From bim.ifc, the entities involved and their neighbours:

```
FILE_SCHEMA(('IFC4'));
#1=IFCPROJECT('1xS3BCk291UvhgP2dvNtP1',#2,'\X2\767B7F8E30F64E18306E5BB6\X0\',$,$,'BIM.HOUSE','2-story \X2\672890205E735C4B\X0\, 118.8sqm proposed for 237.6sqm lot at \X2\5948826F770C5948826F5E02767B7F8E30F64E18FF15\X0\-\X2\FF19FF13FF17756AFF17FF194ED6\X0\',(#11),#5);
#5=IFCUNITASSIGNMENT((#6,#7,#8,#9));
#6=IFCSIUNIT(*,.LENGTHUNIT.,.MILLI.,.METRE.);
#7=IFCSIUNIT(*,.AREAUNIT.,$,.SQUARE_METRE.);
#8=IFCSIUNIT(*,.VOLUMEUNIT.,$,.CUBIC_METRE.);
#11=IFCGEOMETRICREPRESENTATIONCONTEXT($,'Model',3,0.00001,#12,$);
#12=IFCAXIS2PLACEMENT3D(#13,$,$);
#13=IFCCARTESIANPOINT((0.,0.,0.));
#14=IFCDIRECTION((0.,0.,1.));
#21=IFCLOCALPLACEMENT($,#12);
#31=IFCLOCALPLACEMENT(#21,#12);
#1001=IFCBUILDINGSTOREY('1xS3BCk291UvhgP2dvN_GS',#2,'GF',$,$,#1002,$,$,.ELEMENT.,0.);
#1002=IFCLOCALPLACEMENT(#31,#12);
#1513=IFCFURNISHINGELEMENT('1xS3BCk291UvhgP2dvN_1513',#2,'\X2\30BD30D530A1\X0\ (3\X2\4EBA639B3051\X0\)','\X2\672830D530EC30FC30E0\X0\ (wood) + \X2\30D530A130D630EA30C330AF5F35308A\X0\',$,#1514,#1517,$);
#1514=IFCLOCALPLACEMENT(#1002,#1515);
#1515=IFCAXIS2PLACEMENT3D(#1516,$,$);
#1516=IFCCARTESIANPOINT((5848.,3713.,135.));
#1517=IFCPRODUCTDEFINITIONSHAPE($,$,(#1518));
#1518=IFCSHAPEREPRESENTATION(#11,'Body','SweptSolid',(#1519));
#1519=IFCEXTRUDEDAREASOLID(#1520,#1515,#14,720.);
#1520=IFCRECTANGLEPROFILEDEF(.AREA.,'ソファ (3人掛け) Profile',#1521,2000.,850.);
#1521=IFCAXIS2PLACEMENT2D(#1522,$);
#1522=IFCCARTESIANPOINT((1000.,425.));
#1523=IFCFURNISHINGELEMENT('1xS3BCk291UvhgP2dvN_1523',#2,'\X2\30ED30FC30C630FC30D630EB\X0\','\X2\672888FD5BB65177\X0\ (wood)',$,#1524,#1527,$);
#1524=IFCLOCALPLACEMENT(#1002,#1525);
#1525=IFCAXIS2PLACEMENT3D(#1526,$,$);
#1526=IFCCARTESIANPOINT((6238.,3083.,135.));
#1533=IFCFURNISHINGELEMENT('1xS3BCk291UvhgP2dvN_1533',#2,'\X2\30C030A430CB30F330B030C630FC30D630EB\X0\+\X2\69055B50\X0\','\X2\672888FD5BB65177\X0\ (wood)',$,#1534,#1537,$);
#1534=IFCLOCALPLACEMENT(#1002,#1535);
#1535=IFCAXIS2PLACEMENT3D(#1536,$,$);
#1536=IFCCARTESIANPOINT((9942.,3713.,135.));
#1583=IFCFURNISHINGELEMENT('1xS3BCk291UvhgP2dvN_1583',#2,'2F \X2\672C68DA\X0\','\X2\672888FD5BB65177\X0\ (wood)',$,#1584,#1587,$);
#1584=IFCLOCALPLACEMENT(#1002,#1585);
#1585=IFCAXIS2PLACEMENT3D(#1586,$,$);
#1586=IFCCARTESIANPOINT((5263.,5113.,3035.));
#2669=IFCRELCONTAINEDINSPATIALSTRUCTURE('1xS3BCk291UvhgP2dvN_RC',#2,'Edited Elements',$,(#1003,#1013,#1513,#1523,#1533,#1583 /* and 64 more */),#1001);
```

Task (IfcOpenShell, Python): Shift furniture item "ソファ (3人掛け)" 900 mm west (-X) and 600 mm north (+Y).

```python
import ifcopenshell
import ifcopenshell.api.geometry
import ifcopenshell.util.placement
import ifcopenshell.util.unit

model = ifcopenshell.open("bim.ifc")
unit_scale = ifcopenshell.util.unit.calculate_unit_scale(model)

item = model.by_guid("1xS3BCk291UvhgP2dvN_1513")
matrix = ifcopenshell.util.placement.get_local_placement(item.ObjectPlacement)
matrix[0, 3] -= 0.9 / unit_scale
matrix[1, 3] += 0.6 / unit_scale
ifcopenshell.api.geometry.edit_object_placement(model, product=item, matrix=matrix, is_si=False)

print(ifcopenshell.util.placement.get_local_placement(item.ObjectPlacement).round(3) + 0.0)

model.write("bim_rev.ifc")
```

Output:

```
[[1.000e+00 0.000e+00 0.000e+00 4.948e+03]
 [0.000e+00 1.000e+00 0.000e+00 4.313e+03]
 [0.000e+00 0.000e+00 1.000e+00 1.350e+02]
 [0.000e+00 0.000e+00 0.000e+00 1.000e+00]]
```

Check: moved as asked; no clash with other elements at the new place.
